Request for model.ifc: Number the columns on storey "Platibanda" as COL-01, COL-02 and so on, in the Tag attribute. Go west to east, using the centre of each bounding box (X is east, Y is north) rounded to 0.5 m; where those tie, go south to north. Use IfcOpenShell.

First a look at what the model holds.

```python
import ifcopenshell
import ifcopenshell.util.element
import ifcopenshell.util.placement

model = ifcopenshell.open("model.ifc")
print(model.schema)
storey = next(s for s in model.by_type("IfcBuildingStorey") if s.Name == "Platibanda")
columns = [e for e in ifcopenshell.util.element.get_decomposition(storey) if e.is_a("IfcColumn")]
for e in sorted(columns, key=lambda e: e.id()):
    origin = ifcopenshell.util.placement.get_local_placement(e.ObjectPlacement)[:3, 3]
    print(e.id(), e.Tag, e.Name, origin.round(2) + 0.0, sep=" | ")
```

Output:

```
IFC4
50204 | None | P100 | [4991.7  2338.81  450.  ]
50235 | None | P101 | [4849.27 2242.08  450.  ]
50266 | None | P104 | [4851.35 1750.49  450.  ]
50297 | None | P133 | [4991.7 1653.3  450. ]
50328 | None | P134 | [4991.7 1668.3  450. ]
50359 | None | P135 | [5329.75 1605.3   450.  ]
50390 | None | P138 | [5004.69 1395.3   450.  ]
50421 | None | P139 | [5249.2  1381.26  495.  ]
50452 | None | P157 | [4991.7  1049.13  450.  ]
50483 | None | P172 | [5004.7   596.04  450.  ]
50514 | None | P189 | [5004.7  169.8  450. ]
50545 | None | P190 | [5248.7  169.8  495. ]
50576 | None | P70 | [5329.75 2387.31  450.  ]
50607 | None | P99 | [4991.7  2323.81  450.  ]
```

```python
import ifcopenshell
import ifcopenshell.geom
import ifcopenshell.util.element
import ifcopenshell.util.shape

model = ifcopenshell.open("model.ifc")
settings = ifcopenshell.geom.settings()
settings.set("use-world-coords", True)


def centre(element):
    shape = ifcopenshell.geom.create_shape(settings, element)
    return ifcopenshell.util.shape.get_bbox_centroid(shape.geometry)


storey = next(s for s in model.by_type("IfcBuildingStorey") if s.Name == "Platibanda")
columns = [e for e in ifcopenshell.util.element.get_decomposition(storey) if e.is_a("IfcColumn")]

# Insertion points can sit at a corner or the storey origin, so sort by the geometry (in metres).
centres = {e: centre(e) for e in columns}
columns.sort(key=lambda e: (round(centres[e][0] / 0.5), centres[e][1]))

for i, e in enumerate(columns, start=1):
    number = f"COL-{i:02d}"
    e.Tag = number
    print(e.id(), number)

model.write("model-out.ifc")
```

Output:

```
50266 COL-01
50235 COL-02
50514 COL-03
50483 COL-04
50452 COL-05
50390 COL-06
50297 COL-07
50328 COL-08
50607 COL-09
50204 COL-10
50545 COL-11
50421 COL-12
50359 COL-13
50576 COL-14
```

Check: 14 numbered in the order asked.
